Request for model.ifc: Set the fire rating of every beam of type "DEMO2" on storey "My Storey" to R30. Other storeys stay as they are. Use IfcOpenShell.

First a look at what the model holds.

```python
import ifcopenshell
import ifcopenshell.util.element

model = ifcopenshell.open("model.ifc")
print(model.schema)
storey = next(s for s in model.by_type("IfcBuildingStorey") if s.Name == "My Storey")
beams = [e for e in ifcopenshell.util.element.get_decomposition(storey) if e.is_a("IfcBeam")]
seen = {}
for e in beams:
    element_type = ifcopenshell.util.element.get_type(e)
    key = (element_type.Name if element_type != e and element_type else None, ifcopenshell.util.element.get_pset(e, "Pset_BeamCommon", "FireRating"))
    seen[key] = seen.get(key, 0) + 1
for (name, value), count in sorted(seen.items(), key=str):
    print(count, "x", name, "|", value)
```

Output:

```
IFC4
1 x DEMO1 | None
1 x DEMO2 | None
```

```python
import ifcopenshell
import ifcopenshell.api.pset
import ifcopenshell.util.element

model = ifcopenshell.open("model.ifc")

storey = next(s for s in model.by_type("IfcBuildingStorey") if s.Name == "My Storey")
beams = [e for e in ifcopenshell.util.element.get_decomposition(storey) if e.is_a("IfcBeam")]

count = 0
for e in beams:
    element_type = ifcopenshell.util.element.get_type(e)
    if element_type in (None, e) or element_type.Name != "DEMO2":
        continue
    # add_pset returns the element's existing set when there is one.
    pset = ifcopenshell.api.pset.add_pset(model, product=e, name="Pset_BeamCommon")
    ifcopenshell.api.pset.edit_pset(model, pset=pset, properties={"FireRating": "R30"})
    count += 1

print(count, "beams updated")

model.write("model_updated.ifc")
```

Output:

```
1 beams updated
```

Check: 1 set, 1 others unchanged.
